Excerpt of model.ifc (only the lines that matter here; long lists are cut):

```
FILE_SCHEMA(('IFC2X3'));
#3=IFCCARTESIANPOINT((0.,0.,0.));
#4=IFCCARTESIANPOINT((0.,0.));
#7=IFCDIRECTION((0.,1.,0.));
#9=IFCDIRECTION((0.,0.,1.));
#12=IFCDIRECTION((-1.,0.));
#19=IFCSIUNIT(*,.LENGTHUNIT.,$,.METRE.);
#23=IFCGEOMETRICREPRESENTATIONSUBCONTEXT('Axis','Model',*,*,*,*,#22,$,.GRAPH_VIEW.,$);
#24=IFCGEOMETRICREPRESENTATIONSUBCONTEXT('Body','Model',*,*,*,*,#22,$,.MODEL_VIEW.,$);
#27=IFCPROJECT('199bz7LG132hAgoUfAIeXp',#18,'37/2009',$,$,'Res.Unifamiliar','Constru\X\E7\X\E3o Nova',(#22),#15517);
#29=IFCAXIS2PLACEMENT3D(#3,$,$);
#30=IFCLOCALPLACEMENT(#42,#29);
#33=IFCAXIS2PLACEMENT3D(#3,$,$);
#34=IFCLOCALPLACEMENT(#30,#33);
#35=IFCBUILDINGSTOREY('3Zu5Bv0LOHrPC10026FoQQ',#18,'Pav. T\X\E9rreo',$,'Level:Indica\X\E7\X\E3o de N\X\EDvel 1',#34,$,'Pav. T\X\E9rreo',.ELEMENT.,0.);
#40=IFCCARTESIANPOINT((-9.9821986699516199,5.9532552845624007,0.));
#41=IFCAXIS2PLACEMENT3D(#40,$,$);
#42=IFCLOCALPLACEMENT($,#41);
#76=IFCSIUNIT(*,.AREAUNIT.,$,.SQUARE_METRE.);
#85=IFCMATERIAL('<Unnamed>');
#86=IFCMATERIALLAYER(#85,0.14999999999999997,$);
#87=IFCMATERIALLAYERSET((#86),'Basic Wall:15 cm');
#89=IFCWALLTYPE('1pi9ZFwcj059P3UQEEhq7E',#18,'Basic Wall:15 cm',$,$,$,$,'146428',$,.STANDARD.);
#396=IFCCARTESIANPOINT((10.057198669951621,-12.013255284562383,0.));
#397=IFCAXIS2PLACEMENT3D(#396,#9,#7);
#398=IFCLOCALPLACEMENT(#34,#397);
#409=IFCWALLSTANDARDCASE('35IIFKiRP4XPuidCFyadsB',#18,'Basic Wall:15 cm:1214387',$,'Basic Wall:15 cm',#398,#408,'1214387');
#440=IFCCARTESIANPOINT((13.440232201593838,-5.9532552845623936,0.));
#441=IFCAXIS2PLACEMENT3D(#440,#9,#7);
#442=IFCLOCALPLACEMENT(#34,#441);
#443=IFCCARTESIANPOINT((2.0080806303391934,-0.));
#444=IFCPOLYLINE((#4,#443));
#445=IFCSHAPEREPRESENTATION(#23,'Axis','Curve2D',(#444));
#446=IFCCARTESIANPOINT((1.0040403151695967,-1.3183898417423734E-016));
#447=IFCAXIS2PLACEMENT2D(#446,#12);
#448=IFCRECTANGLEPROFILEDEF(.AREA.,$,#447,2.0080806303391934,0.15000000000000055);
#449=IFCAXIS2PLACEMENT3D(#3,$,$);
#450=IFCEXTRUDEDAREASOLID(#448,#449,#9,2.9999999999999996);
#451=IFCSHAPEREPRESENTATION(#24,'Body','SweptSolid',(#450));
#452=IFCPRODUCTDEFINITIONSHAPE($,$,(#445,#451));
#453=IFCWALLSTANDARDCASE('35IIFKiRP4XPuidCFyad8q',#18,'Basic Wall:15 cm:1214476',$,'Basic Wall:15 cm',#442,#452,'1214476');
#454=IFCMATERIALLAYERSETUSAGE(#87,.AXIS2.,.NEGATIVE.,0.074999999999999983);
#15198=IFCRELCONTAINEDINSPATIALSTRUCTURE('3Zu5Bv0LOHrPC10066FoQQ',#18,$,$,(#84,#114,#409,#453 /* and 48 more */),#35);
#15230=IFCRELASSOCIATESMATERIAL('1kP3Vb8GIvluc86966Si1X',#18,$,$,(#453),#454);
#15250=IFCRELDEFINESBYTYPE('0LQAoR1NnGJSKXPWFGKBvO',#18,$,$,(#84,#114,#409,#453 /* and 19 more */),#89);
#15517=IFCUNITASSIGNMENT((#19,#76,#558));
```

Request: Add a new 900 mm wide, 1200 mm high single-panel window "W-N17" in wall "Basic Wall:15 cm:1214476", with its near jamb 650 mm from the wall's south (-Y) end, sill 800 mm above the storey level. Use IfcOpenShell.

```python
import numpy as np
import ifcopenshell
import ifcopenshell.api.feature
import ifcopenshell.api.geometry
import ifcopenshell.api.root
import ifcopenshell.api.spatial
import ifcopenshell.api.type
import ifcopenshell.geom
import ifcopenshell.util.element
import ifcopenshell.util.placement
import ifcopenshell.util.representation
import ifcopenshell.util.shape
import ifcopenshell.util.unit

model = ifcopenshell.open("model.ifc")
unit_scale = ifcopenshell.util.unit.calculate_unit_scale(model)
settings = ifcopenshell.geom.settings()


def volume(element):
    """Net volume in cubic metres, openings subtracted."""
    shape = ifcopenshell.geom.create_shape(settings, element)
    return ifcopenshell.util.shape.get_volume(shape.geometry)


wall = model.by_guid("35IIFKiRP4XPuidCFyad8q")
storey = ifcopenshell.util.element.get_container(wall, ifc_class="IfcBuildingStorey")
context = ifcopenshell.util.representation.get_context(model, "Model", "Body", "MODEL_VIEW")
before = volume(wall)

width, height, from_end, sill = 0.9, 1.2, 0.65, 0.8  # metres

# The wall runs along its own X axis, and the end named is its -X end.
wall_shape = ifcopenshell.geom.create_shape(settings, wall)
x, y, z = ifcopenshell.util.shape.get_vertices(wall_shape.geometry).T
start = x.min() + from_end
face, thickness = float(y.min()), float(y.max() - y.min())
wall_matrix = ifcopenshell.util.placement.get_local_placement(wall.ObjectPlacement)
level = ifcopenshell.util.placement.get_local_placement(storey.ObjectPlacement)[2, 3]


def in_wall(x, y):
    """Placement at x, y metres in the wall's axes, at sill height."""
    matrix = wall_matrix.copy()
    matrix[:, 3] = wall_matrix @ np.array([x / unit_scale, y / unit_scale, 0.0, 1.0])
    matrix[2, 3] = level + sill / unit_scale
    return matrix


# Opening: a box that overshoots both wall faces by 50 mm.
opening = ifcopenshell.api.root.create_entity(model, ifc_class="IfcOpeningElement")
box = ifcopenshell.api.geometry.add_wall_representation(
    model, context=context, length=width, height=height, thickness=thickness + 0.1
)
ifcopenshell.api.geometry.assign_representation(model, product=opening, representation=box)
ifcopenshell.api.geometry.edit_object_placement(model, product=opening, matrix=in_wall(start, face - 0.05), is_si=False)
ifcopenshell.api.feature.add_feature(model, feature=opening, element=wall)

window = ifcopenshell.api.root.create_entity(model, ifc_class="IfcWindow", name="W-N17")
window.OverallWidth, window.OverallHeight = width / unit_scale, height / unit_scale
body = ifcopenshell.api.geometry.add_window_representation(
    model,
    context=context,
    overall_width=window.OverallWidth,
    overall_height=window.OverallHeight,
    partition_type="SINGLE_PANEL",
)
ifcopenshell.api.geometry.assign_representation(model, product=window, representation=body)
ifcopenshell.api.spatial.assign_container(model, products=[window], relating_structure=storey)
fills = ifcopenshell.api.feature.add_filling(model, opening=opening, element=window)
fills.OwnerHistory = window.OwnerHistory  # required in IFC2X3

# IFC2X3 keeps the operation on the window style.
style = ifcopenshell.api.root.create_entity(model, ifc_class="IfcWindowStyle", name="W-N17")
style.OperationType, style.ConstructionType = "SINGLE_PANEL", "NOTDEFINED"
style.ParameterTakesPrecedence = style.Sizeable = False
ifcopenshell.api.type.assign_type(model, related_objects=[window], relating_type=style)

# Centre the window in the wall's thickness.
ifcopenshell.api.geometry.edit_object_placement(model, product=window, matrix=in_wall(start, face), is_si=False)
window_shape = ifcopenshell.geom.create_shape(settings, window)
depth = ifcopenshell.util.shape.get_vertices(window_shape.geometry)[:, 1]
offset = face + thickness / 2 - (depth.min() + depth.max()) / 2
ifcopenshell.api.geometry.edit_object_placement(model, product=window, matrix=in_wall(start, offset), is_si=False)

after = volume(wall)

print(f"wall volume {before:.3f} -> {after:.3f} m3")

model.write("model_v2.ifc")
```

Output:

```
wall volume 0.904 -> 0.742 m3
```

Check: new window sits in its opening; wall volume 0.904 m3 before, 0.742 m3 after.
